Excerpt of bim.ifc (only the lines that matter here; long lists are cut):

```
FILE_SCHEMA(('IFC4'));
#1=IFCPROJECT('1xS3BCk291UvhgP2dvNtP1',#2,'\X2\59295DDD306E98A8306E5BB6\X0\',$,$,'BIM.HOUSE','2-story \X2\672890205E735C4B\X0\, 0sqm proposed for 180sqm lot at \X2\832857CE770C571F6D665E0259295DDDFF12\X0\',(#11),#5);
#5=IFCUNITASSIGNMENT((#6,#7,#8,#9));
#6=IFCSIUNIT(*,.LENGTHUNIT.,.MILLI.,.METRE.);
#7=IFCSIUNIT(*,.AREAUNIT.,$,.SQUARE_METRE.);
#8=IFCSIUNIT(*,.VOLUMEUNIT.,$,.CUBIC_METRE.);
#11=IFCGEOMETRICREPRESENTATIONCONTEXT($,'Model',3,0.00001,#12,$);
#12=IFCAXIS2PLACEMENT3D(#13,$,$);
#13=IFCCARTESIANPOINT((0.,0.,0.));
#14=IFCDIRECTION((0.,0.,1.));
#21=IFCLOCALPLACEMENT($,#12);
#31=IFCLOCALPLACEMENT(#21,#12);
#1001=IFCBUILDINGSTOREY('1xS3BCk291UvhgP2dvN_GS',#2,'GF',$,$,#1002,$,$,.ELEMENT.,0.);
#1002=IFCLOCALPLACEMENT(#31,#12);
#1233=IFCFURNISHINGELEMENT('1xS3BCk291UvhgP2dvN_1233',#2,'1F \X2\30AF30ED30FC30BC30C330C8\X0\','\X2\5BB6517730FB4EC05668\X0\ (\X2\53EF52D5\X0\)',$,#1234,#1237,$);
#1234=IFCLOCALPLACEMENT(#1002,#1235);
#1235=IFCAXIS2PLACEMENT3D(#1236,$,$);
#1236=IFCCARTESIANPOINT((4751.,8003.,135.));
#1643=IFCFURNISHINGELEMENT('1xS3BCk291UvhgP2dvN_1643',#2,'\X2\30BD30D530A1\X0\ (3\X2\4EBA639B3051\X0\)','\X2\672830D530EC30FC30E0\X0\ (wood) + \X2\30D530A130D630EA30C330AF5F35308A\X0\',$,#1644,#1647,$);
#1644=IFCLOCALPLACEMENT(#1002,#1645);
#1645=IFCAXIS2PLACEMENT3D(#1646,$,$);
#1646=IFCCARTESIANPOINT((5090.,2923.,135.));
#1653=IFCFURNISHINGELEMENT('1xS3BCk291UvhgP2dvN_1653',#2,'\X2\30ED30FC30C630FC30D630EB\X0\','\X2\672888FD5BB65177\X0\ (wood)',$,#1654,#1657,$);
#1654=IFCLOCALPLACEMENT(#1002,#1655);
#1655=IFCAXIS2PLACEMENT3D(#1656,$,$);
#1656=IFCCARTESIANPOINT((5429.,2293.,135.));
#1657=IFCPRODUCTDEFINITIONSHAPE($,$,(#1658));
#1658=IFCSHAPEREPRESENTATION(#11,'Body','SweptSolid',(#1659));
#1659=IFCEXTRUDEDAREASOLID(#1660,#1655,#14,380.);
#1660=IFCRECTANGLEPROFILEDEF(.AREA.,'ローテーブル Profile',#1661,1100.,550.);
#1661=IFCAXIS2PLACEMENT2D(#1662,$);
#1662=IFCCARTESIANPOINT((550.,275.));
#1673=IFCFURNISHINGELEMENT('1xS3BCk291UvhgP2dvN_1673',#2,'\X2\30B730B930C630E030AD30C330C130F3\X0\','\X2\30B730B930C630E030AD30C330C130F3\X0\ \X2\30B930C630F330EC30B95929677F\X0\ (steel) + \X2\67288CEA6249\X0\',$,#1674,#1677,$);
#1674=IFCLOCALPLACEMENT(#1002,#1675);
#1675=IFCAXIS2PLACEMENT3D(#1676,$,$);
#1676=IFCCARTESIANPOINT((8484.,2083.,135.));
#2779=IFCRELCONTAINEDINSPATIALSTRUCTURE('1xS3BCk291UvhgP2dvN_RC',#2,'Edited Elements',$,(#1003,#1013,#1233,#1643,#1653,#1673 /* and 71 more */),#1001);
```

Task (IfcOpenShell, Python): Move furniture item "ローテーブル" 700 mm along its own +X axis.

```python
import ifcopenshell
import ifcopenshell.api.geometry
import ifcopenshell.util.placement
import ifcopenshell.util.unit

model = ifcopenshell.open("bim.ifc")
unit_scale = ifcopenshell.util.unit.calculate_unit_scale(model)

item = model.by_id(1653)
matrix = ifcopenshell.util.placement.get_local_placement(item.ObjectPlacement)
matrix[:3, 3] += matrix[:3, 0] * 0.7 / unit_scale
ifcopenshell.api.geometry.edit_object_placement(model, product=item, matrix=matrix, is_si=False)

print(ifcopenshell.util.placement.get_local_placement(item.ObjectPlacement).round(3) + 0.0)

model.write("bim_v2.ifc")
```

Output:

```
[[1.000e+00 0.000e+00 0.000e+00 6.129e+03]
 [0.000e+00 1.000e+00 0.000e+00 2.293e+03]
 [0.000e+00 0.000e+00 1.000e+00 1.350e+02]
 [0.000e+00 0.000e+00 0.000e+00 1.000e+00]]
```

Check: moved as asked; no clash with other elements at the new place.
